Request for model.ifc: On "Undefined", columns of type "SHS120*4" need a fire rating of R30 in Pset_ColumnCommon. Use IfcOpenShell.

First a look at what the model holds.

```python
import ifcopenshell
import ifcopenshell.util.element

model = ifcopenshell.open("model.ifc")
print(model.schema)
storey = next(s for s in model.by_type("IfcBuildingStorey") if s.Name == "Undefined")
columns = [e for e in ifcopenshell.util.element.get_decomposition(storey) if e.is_a("IfcColumn")]
seen = {}
for e in columns:
    element_type = ifcopenshell.util.element.get_type(e)
    key = (element_type.Name if element_type != e and element_type else None, ifcopenshell.util.element.get_pset(e, "Pset_ColumnCommon", "FireRating"))
    seen[key] = seen.get(key, 0) + 1
for (name, value), count in sorted(seen.items(), key=str):
    print(count, "x", name, "|", value)
```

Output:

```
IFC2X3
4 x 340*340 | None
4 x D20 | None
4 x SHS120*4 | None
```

```python
import ifcopenshell
import ifcopenshell.api.pset
import ifcopenshell.util.element

model = ifcopenshell.open("model.ifc")

storey = next(s for s in model.by_type("IfcBuildingStorey") if s.Name == "Undefined")
columns = [e for e in ifcopenshell.util.element.get_decomposition(storey) if e.is_a("IfcColumn")]

count = 0
for e in columns:
    element_type = ifcopenshell.util.element.get_type(e)
    if element_type in (None, e) or element_type.Name != "SHS120*4":
        continue
    # add_pset returns the element's existing set when there is one.
    pset = ifcopenshell.api.pset.add_pset(model, product=e, name="Pset_ColumnCommon")
    ifcopenshell.api.pset.edit_pset(model, pset=pset, properties={"FireRating": "R30"})
    count += 1

print(count, "columns updated")

model.write("model_v2.ifc")
```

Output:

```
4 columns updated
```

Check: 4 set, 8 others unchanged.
